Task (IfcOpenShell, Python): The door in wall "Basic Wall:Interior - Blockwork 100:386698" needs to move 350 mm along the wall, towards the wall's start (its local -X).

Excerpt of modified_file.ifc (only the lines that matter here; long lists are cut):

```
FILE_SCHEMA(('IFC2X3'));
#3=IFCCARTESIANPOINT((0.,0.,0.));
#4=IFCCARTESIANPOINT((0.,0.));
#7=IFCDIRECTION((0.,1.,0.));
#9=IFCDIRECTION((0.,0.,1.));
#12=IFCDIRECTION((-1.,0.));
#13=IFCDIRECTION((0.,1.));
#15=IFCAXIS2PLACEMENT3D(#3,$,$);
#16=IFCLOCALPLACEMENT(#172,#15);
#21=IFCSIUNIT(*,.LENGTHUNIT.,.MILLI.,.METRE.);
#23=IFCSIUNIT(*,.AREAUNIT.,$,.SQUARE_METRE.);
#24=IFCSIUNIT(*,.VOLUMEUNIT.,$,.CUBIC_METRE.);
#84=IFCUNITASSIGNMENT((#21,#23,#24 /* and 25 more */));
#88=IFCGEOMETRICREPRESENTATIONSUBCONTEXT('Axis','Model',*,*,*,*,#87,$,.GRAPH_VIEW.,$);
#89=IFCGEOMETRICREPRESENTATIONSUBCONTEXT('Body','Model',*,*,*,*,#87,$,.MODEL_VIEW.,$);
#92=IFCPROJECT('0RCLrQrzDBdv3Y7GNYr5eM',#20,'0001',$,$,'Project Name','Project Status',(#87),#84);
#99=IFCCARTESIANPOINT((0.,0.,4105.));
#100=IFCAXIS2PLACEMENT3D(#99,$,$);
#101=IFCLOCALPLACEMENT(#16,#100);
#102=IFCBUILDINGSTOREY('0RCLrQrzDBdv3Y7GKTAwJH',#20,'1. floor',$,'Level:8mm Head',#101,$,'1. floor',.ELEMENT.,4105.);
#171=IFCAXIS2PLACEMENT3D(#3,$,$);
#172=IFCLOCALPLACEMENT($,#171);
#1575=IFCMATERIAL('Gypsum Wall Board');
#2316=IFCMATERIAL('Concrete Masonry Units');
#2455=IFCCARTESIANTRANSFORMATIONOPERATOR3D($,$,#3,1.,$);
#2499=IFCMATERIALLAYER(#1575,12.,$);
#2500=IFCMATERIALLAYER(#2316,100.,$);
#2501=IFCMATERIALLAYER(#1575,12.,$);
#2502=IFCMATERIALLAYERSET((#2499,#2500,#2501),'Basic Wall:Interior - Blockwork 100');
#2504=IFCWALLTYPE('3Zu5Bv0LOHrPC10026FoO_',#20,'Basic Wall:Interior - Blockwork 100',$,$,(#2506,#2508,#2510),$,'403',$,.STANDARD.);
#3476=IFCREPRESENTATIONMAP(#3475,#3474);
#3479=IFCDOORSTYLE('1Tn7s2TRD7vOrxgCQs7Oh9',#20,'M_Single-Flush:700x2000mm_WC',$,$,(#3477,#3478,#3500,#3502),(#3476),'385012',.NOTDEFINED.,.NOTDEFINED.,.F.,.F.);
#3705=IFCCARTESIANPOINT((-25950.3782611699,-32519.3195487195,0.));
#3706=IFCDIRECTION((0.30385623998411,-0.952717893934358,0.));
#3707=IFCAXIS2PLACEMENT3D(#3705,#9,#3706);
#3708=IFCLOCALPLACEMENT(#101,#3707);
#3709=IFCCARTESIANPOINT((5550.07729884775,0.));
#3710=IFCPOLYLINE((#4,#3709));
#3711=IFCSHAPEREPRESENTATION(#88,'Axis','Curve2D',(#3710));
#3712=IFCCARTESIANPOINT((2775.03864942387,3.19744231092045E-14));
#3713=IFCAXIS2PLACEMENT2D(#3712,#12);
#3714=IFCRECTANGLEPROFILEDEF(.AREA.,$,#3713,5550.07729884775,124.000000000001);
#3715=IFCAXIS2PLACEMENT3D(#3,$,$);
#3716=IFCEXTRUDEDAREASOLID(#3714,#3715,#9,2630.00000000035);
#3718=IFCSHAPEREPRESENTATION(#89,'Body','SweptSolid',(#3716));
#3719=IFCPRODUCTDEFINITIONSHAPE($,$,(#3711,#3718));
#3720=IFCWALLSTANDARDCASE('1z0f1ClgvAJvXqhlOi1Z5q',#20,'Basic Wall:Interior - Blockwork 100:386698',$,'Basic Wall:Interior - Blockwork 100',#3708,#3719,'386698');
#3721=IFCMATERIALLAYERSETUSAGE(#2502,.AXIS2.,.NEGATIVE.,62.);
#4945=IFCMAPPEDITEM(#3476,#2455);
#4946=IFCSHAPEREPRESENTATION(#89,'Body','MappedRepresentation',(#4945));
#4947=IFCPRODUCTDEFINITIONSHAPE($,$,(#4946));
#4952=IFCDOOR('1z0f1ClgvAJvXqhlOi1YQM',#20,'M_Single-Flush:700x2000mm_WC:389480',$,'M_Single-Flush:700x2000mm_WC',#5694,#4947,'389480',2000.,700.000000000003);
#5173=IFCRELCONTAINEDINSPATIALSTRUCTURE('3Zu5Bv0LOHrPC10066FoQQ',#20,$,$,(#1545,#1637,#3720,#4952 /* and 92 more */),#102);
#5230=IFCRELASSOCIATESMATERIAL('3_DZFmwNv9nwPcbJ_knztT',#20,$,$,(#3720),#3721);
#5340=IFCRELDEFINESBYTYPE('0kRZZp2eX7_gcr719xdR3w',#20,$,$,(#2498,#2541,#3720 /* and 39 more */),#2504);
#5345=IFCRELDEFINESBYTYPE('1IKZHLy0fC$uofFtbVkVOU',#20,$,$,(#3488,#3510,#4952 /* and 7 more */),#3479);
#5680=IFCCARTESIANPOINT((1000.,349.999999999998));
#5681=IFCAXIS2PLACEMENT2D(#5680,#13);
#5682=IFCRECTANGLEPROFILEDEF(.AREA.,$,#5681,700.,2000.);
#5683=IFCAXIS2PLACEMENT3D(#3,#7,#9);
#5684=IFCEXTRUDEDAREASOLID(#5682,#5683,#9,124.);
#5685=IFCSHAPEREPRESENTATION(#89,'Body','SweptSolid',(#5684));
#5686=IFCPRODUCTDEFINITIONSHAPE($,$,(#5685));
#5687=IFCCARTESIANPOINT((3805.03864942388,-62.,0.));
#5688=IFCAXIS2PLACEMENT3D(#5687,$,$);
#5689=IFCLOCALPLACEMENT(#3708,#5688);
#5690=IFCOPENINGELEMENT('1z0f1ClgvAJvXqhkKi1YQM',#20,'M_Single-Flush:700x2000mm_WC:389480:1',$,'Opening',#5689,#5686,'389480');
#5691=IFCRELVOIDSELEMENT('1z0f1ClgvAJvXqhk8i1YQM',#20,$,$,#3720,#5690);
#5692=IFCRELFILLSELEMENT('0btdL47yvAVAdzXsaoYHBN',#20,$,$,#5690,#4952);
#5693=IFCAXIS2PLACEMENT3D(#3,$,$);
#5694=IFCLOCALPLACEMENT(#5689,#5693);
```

```python
import ifcopenshell
import ifcopenshell.api.geometry
import ifcopenshell.util.placement
import ifcopenshell.util.unit

model = ifcopenshell.open("modified_file.ifc")
unit_scale = ifcopenshell.util.unit.calculate_unit_scale(model)

door = model.by_guid("1z0f1ClgvAJvXqhlOi1YQM")
opening = door.FillsVoids[0].RelatingOpeningElement
wall = opening.VoidsElements[0].RelatingBuildingElement

wall_matrix = ifcopenshell.util.placement.get_local_placement(wall.ObjectPlacement)
shift = wall_matrix[:3, 0] * -0.35 / unit_scale
before = ifcopenshell.util.placement.get_local_placement(door.ObjectPlacement)[:3, 3].copy()

# The door is placed relative to its opening, so it follows when the opening moves.
matrix = ifcopenshell.util.placement.get_local_placement(opening.ObjectPlacement)
matrix[:3, 3] += shift
ifcopenshell.api.geometry.edit_object_placement(
    model, product=opening, matrix=matrix, is_si=False, should_transform_children=True
)

after = ifcopenshell.util.placement.get_local_placement(door.ObjectPlacement)[:3, 3]
print("door moved by", (after - before).round(3) + 0.0)

model.write("modified_file-out.ifc")
```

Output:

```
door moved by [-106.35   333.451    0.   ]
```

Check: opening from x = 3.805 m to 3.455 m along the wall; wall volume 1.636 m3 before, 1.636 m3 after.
